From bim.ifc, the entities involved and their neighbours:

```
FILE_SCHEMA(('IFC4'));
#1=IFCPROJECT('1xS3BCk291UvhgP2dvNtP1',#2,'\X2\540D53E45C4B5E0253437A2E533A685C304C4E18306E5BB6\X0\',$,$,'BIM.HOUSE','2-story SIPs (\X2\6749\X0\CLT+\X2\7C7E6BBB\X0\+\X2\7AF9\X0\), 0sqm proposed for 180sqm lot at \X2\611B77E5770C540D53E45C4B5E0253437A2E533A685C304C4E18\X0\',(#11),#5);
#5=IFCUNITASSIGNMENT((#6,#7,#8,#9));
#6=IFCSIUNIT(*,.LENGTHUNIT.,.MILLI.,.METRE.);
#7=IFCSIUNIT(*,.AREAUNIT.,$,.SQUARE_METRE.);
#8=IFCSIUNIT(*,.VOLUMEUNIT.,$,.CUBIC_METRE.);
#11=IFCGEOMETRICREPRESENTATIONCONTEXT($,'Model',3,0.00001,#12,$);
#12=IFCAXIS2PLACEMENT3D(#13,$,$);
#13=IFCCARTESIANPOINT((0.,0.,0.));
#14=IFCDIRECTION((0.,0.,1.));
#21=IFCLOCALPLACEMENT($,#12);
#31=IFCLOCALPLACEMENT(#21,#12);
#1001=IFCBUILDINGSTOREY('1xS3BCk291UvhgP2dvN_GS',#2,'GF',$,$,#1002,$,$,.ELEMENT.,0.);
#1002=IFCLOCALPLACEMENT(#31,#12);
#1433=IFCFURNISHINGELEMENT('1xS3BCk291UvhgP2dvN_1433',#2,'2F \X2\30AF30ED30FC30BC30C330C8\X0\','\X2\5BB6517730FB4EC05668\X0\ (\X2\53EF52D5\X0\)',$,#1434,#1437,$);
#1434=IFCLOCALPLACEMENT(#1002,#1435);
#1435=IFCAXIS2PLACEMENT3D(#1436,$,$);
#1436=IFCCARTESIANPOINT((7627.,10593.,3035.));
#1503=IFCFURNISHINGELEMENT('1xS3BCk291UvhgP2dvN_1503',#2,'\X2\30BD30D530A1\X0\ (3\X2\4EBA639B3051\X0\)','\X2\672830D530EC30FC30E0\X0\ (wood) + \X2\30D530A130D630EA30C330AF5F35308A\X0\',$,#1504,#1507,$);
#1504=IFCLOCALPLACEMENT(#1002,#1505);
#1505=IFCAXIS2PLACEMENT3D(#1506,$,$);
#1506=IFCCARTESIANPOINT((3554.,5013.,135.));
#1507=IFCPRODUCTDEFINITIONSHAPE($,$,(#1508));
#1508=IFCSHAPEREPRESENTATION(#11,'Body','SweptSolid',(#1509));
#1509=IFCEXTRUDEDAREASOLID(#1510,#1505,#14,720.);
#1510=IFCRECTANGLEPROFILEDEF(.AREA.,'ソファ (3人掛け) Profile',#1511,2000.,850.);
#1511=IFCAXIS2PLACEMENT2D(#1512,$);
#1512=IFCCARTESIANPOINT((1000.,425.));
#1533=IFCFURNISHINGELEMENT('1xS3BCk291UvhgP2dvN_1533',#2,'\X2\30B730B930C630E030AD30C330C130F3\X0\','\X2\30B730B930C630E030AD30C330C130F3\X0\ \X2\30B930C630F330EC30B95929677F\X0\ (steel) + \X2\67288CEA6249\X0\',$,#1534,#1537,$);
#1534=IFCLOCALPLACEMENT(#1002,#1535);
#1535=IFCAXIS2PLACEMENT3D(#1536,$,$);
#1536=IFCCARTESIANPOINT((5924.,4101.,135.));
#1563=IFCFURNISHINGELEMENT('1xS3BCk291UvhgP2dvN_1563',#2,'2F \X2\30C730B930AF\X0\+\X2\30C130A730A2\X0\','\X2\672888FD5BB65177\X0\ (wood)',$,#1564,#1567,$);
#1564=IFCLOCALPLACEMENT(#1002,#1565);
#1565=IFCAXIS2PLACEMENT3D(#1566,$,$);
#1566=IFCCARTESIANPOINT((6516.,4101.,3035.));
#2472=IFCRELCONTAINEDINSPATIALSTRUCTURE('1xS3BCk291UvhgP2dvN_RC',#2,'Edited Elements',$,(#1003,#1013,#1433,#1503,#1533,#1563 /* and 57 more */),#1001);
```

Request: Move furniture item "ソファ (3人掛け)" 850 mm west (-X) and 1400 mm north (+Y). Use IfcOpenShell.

```python
import ifcopenshell
import ifcopenshell.api.geometry
import ifcopenshell.util.placement

model = ifcopenshell.open("bim.ifc")

item = model.by_guid("1xS3BCk291UvhgP2dvN_1503")
matrix = ifcopenshell.util.placement.get_local_placement(item.ObjectPlacement)
matrix[0, 3] -= 850.0
matrix[1, 3] += 1400.0
ifcopenshell.api.geometry.edit_object_placement(model, product=item, matrix=matrix, is_si=False)

print(ifcopenshell.util.placement.get_local_placement(item.ObjectPlacement).round(3) + 0.0)

model.write("bim_edited.ifc")
```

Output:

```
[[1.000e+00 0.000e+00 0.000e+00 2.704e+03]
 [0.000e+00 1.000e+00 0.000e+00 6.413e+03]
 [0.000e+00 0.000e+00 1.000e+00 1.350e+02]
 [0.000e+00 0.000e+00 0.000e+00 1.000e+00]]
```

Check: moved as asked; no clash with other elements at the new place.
